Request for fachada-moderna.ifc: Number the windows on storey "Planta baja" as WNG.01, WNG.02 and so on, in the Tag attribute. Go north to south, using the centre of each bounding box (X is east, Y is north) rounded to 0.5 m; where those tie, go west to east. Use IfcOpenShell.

First a look at what the model holds.

```python
import ifcopenshell
import ifcopenshell.util.element
import ifcopenshell.util.placement

model = ifcopenshell.open("fachada-moderna.ifc")
print(model.schema)
storey = next(s for s in model.by_type("IfcBuildingStorey") if s.Name == "Planta baja")
windows = [e for e in ifcopenshell.util.element.get_decomposition(storey) if e.is_a("IfcWindow")]
for e in sorted(windows, key=lambda e: e.id()):
    origin = ifcopenshell.util.placement.get_local_placement(e.ObjectPlacement)[:3, 3]
    print(e.id(), e.Tag, e.Name, origin.round(2) + 0.0, sep=" | ")
```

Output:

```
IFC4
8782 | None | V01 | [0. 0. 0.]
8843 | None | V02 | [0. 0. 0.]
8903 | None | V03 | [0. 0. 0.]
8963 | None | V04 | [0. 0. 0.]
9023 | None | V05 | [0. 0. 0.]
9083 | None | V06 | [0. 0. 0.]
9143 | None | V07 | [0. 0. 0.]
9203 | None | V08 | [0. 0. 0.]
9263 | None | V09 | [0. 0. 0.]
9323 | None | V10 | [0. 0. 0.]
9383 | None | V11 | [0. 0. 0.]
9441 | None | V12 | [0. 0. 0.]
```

```python
import ifcopenshell
import ifcopenshell.geom
import ifcopenshell.util.element
import ifcopenshell.util.shape

model = ifcopenshell.open("fachada-moderna.ifc")
settings = ifcopenshell.geom.settings()
settings.set("use-world-coords", True)


def centre(element):
    shape = ifcopenshell.geom.create_shape(settings, element)
    return ifcopenshell.util.shape.get_bbox_centroid(shape.geometry)


storey = next(s for s in model.by_type("IfcBuildingStorey") if s.Name == "Planta baja")
windows = [e for e in ifcopenshell.util.element.get_decomposition(storey) if e.is_a("IfcWindow")]

# Insertion points can sit at a corner or the storey origin, so sort by the geometry (in metres).
centres = {e: centre(e) for e in windows}
windows.sort(key=lambda e: (-round(centres[e][1] / 0.5), centres[e][0]))

for i, e in enumerate(windows, start=1):
    number = f"WNG.{i:02d}"
    e.Tag = number
    print(e.id(), number)

model.write("fachada-moderna_updated.ifc")
```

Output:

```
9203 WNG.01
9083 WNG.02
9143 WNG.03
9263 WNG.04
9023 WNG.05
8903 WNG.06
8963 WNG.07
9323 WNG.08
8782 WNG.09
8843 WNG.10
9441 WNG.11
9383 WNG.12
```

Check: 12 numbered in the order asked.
